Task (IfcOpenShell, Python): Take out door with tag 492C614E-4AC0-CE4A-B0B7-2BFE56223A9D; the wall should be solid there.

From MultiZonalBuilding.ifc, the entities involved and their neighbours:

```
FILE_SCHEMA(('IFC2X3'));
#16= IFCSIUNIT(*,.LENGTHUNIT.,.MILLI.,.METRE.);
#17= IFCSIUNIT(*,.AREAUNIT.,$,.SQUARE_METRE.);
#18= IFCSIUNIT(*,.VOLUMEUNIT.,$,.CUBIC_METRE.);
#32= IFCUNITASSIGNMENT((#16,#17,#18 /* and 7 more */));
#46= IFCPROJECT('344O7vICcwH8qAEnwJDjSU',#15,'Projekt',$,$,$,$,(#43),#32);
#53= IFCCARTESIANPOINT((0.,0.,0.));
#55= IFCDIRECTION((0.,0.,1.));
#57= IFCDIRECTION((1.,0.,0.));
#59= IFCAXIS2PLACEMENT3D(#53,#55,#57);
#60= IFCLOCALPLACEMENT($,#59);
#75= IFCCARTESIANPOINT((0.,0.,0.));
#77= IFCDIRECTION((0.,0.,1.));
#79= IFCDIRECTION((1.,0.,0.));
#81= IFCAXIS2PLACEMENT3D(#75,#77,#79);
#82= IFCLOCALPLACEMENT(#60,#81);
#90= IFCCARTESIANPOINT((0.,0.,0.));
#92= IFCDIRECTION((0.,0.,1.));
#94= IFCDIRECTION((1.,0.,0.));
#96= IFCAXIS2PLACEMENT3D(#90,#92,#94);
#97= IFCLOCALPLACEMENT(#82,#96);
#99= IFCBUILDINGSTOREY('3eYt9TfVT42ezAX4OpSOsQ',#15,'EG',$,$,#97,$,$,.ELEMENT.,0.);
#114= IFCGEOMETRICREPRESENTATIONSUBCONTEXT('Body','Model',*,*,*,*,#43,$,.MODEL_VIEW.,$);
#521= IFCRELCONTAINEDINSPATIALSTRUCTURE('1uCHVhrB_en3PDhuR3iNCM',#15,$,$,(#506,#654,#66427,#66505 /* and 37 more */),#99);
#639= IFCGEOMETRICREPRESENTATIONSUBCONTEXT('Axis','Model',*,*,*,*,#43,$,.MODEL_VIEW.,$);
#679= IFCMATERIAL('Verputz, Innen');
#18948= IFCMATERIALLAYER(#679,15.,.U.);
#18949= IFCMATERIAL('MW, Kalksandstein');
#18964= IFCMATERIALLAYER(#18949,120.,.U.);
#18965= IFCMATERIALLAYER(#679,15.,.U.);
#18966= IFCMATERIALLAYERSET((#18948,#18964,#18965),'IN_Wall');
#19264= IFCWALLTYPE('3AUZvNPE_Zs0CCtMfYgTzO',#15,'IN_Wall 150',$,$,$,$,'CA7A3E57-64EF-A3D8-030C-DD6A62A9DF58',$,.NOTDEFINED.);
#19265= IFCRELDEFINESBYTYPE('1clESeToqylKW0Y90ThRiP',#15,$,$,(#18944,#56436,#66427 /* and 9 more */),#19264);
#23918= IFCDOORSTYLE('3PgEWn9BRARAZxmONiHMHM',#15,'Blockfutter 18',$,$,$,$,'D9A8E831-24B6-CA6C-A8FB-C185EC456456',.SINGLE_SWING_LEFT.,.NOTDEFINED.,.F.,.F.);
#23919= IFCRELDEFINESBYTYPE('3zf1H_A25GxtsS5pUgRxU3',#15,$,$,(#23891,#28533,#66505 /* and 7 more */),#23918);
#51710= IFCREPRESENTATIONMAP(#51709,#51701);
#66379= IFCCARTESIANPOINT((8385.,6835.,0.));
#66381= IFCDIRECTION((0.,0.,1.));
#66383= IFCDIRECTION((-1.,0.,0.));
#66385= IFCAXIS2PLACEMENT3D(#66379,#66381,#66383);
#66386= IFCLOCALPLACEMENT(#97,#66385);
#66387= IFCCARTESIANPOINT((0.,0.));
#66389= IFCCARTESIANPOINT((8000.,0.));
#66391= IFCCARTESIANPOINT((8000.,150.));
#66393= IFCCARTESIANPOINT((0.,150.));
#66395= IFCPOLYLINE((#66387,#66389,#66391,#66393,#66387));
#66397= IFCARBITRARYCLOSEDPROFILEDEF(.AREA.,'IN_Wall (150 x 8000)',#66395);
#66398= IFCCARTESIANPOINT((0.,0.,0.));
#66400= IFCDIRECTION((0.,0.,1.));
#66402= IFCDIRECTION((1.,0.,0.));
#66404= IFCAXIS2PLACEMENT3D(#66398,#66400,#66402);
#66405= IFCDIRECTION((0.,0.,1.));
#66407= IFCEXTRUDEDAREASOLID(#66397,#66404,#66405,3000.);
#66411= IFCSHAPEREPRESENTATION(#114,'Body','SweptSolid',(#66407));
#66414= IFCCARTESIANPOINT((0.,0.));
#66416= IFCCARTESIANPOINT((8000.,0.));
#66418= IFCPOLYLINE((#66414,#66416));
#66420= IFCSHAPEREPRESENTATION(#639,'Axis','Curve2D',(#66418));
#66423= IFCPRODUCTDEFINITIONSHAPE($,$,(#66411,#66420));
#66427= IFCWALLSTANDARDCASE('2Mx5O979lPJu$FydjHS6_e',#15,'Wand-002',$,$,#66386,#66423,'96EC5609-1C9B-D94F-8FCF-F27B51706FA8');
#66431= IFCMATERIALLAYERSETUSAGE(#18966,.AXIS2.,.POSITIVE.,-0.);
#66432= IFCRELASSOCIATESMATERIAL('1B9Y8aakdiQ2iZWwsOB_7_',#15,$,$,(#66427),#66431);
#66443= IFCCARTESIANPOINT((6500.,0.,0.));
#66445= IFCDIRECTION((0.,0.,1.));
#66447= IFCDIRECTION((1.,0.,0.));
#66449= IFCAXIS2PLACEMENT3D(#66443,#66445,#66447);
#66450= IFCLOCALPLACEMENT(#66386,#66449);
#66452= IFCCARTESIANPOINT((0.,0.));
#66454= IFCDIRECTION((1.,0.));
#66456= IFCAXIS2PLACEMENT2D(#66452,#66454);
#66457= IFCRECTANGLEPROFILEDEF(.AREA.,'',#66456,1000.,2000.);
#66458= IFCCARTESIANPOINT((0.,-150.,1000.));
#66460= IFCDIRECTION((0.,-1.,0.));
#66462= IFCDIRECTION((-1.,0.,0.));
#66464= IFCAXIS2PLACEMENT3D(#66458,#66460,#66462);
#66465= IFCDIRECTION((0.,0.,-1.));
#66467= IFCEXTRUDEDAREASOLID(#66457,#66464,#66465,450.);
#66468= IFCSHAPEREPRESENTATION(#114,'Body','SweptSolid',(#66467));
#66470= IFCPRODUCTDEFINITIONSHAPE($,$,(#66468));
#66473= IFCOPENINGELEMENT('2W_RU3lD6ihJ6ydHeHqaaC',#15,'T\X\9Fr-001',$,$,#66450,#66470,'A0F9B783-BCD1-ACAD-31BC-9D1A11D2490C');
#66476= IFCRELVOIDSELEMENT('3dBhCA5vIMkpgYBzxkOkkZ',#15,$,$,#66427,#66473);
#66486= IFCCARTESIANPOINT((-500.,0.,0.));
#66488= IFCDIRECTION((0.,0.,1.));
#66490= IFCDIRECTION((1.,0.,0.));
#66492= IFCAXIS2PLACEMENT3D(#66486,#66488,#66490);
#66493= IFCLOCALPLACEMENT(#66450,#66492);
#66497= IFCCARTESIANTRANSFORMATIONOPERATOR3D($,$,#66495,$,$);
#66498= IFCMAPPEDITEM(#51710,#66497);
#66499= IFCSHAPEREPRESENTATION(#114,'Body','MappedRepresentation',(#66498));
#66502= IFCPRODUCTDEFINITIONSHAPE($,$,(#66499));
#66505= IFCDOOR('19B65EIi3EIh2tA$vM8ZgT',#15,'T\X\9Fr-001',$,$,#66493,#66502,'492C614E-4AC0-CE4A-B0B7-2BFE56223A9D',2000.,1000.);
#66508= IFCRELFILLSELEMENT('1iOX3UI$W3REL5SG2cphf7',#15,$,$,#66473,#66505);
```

```python
import ifcopenshell
import ifcopenshell.api.feature
import ifcopenshell.api.root
import ifcopenshell.geom
import ifcopenshell.util.shape

model = ifcopenshell.open("MultiZonalBuilding.ifc")
settings = ifcopenshell.geom.settings()


def volume(element):
    """Net volume in cubic metres, openings subtracted."""
    shape = ifcopenshell.geom.create_shape(settings, element)
    return ifcopenshell.util.shape.get_volume(shape.geometry)


door = model.by_id(66505)
opening = door.FillsVoids[0].RelatingOpeningElement
wall = opening.VoidsElements[0].RelatingBuildingElement
before = volume(wall)

ifcopenshell.api.root.remove_product(model, product=door)
ifcopenshell.api.feature.remove_feature(model, feature=opening)

after = volume(wall)

print(f"wall volume {before:.3f} -> {after:.3f} m3")

model.write("MultiZonalBuilding_v2.ifc")
```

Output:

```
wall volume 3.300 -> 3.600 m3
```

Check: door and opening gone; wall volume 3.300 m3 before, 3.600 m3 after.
